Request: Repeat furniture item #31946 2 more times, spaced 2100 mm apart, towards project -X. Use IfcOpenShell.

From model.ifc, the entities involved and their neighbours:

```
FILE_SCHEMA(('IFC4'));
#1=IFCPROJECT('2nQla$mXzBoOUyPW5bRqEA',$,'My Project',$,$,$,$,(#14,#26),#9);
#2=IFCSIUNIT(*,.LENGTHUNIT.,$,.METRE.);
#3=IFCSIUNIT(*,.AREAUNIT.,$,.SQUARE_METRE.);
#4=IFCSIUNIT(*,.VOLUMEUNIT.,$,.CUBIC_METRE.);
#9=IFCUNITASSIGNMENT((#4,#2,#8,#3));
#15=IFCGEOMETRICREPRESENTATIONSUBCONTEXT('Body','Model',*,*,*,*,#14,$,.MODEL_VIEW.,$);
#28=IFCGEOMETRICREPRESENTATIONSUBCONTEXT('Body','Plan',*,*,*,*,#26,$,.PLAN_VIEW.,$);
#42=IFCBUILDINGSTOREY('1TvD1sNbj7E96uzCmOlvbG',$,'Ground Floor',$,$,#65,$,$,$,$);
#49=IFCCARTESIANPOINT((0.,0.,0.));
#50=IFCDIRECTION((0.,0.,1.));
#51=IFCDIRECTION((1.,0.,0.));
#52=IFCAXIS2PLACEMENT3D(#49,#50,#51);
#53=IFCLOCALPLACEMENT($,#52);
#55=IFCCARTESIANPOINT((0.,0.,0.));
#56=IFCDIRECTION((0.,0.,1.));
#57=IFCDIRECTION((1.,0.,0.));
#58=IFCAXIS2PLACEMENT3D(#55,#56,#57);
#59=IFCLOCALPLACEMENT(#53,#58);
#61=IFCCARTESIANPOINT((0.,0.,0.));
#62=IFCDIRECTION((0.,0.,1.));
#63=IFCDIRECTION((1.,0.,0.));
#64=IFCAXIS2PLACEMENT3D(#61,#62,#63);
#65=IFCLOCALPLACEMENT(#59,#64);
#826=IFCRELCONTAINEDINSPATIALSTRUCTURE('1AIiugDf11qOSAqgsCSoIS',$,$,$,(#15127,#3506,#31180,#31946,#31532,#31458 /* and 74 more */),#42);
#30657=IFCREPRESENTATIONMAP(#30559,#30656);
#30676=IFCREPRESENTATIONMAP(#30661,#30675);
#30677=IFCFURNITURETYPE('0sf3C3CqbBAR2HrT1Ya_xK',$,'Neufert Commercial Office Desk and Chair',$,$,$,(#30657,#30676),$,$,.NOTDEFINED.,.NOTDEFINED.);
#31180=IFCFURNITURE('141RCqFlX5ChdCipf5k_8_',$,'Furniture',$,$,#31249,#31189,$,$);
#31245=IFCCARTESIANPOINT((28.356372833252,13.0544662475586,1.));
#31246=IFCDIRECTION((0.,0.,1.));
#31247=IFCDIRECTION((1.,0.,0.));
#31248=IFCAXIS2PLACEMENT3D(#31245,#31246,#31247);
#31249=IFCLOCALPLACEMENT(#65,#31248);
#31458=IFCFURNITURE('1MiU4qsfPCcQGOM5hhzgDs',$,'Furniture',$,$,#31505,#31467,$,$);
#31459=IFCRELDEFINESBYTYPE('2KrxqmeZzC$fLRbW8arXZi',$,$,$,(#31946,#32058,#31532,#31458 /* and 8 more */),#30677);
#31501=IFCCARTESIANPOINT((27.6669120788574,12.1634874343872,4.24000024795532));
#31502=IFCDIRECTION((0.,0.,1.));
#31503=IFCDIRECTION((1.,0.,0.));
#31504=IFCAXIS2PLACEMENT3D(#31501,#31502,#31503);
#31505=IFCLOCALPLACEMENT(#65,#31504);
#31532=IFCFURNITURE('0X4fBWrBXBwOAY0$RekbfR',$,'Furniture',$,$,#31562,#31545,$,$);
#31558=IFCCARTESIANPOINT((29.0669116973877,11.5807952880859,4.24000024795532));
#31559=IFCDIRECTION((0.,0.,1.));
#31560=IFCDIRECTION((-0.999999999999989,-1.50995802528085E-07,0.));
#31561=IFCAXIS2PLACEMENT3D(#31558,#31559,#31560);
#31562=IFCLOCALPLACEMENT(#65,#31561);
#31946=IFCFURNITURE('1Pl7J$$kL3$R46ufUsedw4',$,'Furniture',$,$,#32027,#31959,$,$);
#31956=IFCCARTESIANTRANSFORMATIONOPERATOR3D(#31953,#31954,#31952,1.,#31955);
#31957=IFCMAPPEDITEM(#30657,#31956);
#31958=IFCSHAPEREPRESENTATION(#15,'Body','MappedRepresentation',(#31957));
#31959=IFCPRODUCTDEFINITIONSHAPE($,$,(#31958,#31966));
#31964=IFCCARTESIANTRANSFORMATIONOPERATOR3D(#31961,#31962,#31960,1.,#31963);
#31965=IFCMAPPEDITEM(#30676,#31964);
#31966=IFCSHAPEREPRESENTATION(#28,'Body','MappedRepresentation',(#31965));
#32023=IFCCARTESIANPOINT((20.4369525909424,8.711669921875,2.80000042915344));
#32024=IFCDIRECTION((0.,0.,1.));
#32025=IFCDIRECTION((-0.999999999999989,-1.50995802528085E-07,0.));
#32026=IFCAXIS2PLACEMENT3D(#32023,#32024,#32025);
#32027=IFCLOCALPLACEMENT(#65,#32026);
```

```python
import numpy as np
import ifcopenshell
import ifcopenshell.api.geometry
import ifcopenshell.api.root
import ifcopenshell.util.element
import ifcopenshell.util.placement

model = ifcopenshell.open("model.ifc")

source = model.by_guid("1Pl7J$$kL3$R46ufUsedw4")
base = ifcopenshell.util.placement.get_local_placement(source.ObjectPlacement)
step = np.array([-1.0, 0.0, 0.0]) * 2.1

for i in range(1, 3):
    copy = ifcopenshell.api.root.copy_class(model, product=source)
    copy.Representation = ifcopenshell.util.element.copy_deep(
        model, source.Representation, exclude=["IfcGeometricRepresentationContext", "IfcRepresentationMap"]
    )
    matrix = base.copy()
    matrix[:3, 3] += i * step
    print("added at", matrix[:3, 3].round(3) + 0.0)
    ifcopenshell.api.geometry.edit_object_placement(model, product=copy, matrix=matrix, is_si=False)

model.write("model-out.ifc")
```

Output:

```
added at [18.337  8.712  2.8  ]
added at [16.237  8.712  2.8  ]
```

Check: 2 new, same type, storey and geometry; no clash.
